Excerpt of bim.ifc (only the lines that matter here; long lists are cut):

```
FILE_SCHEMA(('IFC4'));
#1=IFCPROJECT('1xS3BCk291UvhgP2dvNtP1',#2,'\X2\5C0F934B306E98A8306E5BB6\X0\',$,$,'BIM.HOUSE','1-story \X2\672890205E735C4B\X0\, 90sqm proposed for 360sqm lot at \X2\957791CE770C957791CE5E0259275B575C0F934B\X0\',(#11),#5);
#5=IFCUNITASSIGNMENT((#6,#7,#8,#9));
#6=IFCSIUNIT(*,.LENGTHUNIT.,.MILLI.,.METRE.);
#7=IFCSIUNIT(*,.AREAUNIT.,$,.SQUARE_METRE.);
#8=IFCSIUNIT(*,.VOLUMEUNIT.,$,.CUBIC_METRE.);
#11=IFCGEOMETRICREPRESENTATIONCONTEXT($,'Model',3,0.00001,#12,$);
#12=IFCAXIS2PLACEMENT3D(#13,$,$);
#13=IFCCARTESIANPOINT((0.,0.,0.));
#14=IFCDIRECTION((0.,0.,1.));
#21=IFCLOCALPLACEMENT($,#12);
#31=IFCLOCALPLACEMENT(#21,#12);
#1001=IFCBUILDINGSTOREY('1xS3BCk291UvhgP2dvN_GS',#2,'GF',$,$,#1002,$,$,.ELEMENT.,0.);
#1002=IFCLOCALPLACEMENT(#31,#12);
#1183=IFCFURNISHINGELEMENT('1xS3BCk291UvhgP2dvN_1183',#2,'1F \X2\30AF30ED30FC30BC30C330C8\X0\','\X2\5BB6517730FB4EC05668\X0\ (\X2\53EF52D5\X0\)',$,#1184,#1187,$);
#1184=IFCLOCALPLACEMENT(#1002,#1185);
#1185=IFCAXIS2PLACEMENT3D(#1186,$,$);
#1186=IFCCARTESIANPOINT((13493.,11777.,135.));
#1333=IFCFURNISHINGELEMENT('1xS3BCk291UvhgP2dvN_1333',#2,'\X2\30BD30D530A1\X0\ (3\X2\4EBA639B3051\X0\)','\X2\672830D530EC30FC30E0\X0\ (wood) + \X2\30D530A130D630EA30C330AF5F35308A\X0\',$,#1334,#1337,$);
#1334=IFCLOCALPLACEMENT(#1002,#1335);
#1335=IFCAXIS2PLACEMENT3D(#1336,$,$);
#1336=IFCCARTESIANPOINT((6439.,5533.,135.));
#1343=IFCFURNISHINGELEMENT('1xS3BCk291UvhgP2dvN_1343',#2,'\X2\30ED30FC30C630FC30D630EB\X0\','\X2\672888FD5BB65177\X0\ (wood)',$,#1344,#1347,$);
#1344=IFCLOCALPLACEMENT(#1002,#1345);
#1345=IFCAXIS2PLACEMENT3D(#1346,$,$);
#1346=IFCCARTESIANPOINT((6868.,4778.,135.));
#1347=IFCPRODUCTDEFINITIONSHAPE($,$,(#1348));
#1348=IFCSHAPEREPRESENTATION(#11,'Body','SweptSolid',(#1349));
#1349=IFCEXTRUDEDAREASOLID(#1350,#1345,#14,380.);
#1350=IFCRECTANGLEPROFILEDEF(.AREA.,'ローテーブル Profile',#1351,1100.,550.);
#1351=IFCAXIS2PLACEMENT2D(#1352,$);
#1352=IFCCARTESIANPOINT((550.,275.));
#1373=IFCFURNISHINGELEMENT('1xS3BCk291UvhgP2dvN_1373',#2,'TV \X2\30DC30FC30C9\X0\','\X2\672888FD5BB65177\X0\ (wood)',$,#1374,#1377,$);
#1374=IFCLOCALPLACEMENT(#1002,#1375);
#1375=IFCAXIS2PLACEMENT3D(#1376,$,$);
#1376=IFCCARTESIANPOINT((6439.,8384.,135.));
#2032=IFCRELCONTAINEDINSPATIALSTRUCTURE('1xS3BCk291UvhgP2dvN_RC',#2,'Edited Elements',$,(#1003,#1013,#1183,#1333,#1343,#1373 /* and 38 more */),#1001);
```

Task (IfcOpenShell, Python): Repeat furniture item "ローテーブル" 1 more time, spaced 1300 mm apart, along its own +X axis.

```python
import ifcopenshell
import ifcopenshell.api.geometry
import ifcopenshell.api.root
import ifcopenshell.util.element
import ifcopenshell.util.placement
import ifcopenshell.util.unit

model = ifcopenshell.open("bim.ifc")
unit_scale = ifcopenshell.util.unit.calculate_unit_scale(model)


def reuse_history(source, copy):
    """copy_class also copies each property set's owner history, people and application; keep the originals."""
    for rel in copy.IsDefinedBy:
        if rel.is_a("IfcRelDefinesByProperties") and (history := rel.RelatingPropertyDefinition.OwnerHistory):
            rel.RelatingPropertyDefinition.OwnerHistory = source.OwnerHistory
            ifcopenshell.util.element.remove_deep2(model, history)


source = model.by_id(1343)
base = ifcopenshell.util.placement.get_local_placement(source.ObjectPlacement)
step = base[:3, 0] * 1.3 / unit_scale

for i in range(1, 2):
    copy = ifcopenshell.api.root.copy_class(model, product=source)
    copy.Representation = ifcopenshell.util.element.copy_deep(
        model, source.Representation, exclude=["IfcGeometricRepresentationContext", "IfcRepresentationMap"]
    )
    reuse_history(source, copy)
    matrix = base.copy()
    matrix[:3, 3] += i * step
    print("added at", matrix[:3, 3].round(3) + 0.0)
    ifcopenshell.api.geometry.edit_object_placement(model, product=copy, matrix=matrix, is_si=False)

model.write("bim_v2.ifc")
```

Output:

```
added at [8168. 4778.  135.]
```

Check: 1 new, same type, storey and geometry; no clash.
